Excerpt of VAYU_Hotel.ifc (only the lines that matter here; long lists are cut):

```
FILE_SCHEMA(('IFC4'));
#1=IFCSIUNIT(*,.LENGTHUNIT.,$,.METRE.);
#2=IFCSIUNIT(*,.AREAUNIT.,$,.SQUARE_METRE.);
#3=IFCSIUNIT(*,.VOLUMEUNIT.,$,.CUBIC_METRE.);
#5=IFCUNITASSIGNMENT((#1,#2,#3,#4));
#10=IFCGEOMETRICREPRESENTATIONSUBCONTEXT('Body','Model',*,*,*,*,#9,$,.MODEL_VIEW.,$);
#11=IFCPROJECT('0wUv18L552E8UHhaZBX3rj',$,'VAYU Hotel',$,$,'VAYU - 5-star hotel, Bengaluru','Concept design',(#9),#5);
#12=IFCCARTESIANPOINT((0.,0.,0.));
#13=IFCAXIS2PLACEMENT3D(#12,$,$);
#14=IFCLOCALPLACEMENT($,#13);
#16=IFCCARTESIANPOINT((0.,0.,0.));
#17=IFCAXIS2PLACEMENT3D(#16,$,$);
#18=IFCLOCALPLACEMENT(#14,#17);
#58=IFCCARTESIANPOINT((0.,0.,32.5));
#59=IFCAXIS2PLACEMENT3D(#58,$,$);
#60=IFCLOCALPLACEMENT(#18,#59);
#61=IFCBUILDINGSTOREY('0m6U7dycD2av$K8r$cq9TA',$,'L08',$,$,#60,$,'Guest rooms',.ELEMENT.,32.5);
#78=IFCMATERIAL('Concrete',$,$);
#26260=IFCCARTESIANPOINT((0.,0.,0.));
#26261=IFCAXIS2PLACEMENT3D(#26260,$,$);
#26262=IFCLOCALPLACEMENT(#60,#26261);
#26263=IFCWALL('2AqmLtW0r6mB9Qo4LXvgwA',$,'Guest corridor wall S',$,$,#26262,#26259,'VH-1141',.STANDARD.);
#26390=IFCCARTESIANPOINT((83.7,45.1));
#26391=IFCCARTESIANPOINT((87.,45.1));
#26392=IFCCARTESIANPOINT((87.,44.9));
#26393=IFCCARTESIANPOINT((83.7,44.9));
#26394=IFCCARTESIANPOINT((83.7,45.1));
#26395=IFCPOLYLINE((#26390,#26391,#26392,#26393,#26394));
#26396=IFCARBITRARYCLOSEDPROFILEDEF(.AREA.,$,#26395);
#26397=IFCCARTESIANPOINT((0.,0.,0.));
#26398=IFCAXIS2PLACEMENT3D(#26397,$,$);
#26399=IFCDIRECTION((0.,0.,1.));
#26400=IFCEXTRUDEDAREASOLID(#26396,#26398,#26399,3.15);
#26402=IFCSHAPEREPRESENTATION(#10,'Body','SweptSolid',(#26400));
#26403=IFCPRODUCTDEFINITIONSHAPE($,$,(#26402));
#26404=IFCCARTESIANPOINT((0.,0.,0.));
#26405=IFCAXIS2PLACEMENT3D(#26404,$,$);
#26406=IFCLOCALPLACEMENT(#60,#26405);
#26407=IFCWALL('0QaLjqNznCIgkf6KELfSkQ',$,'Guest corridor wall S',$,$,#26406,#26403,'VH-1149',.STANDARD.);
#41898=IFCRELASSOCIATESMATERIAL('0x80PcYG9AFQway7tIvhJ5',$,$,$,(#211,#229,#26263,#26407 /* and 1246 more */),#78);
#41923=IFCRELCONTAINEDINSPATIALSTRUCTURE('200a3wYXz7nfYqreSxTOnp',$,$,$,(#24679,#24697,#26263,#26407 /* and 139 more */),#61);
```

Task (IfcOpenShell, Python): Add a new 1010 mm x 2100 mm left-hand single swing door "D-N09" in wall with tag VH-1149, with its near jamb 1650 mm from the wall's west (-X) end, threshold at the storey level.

```python
import numpy as np
import ifcopenshell
import ifcopenshell.api.feature
import ifcopenshell.api.geometry
import ifcopenshell.api.root
import ifcopenshell.api.spatial
import ifcopenshell.geom
import ifcopenshell.util.element
import ifcopenshell.util.placement
import ifcopenshell.util.representation
import ifcopenshell.util.shape
import ifcopenshell.util.unit

model = ifcopenshell.open("VAYU_Hotel.ifc")
unit_scale = ifcopenshell.util.unit.calculate_unit_scale(model)
settings = ifcopenshell.geom.settings()


def volume(element):
    """Net volume in cubic metres, openings subtracted."""
    shape = ifcopenshell.geom.create_shape(settings, element)
    return ifcopenshell.util.shape.get_volume(shape.geometry)


wall = model.by_guid("0QaLjqNznCIgkf6KELfSkQ")
storey = ifcopenshell.util.element.get_container(wall, ifc_class="IfcBuildingStorey")
context = ifcopenshell.util.representation.get_context(model, "Model", "Body", "MODEL_VIEW")
before = volume(wall)

width, height, from_end, sill = 1.01, 2.1, 1.65, 0.0  # metres

# The wall runs along its own X axis, and the end named is its -X end.
wall_shape = ifcopenshell.geom.create_shape(settings, wall)
x, y, z = ifcopenshell.util.shape.get_vertices(wall_shape.geometry).T
start = x.min() + from_end
face, thickness = float(y.min()), float(y.max() - y.min())
wall_matrix = ifcopenshell.util.placement.get_local_placement(wall.ObjectPlacement)
level = ifcopenshell.util.placement.get_local_placement(storey.ObjectPlacement)[2, 3]


def in_wall(x, y):
    """Placement at x, y metres in the wall's axes, at sill height."""
    matrix = wall_matrix.copy()
    matrix[:, 3] = wall_matrix @ np.array([x / unit_scale, y / unit_scale, 0.0, 1.0])
    matrix[2, 3] = level + sill / unit_scale
    return matrix


# Opening: a box that overshoots both wall faces by 50 mm.
opening = ifcopenshell.api.root.create_entity(model, ifc_class="IfcOpeningElement", predefined_type="OPENING")
box = ifcopenshell.api.geometry.add_wall_representation(
    model, context=context, length=width, height=height, thickness=thickness + 0.1
)
ifcopenshell.api.geometry.assign_representation(model, product=opening, representation=box)
ifcopenshell.api.geometry.edit_object_placement(model, product=opening, matrix=in_wall(start, face - 0.05), is_si=False)
ifcopenshell.api.feature.add_feature(model, feature=opening, element=wall)

door = ifcopenshell.api.root.create_entity(model, ifc_class="IfcDoor", name="D-N09", predefined_type="DOOR")
door.OverallWidth, door.OverallHeight = width / unit_scale, height / unit_scale
door.OperationType = "SINGLE_SWING_LEFT"
body = ifcopenshell.api.geometry.add_door_representation(
    model,
    context=context,
    overall_width=door.OverallWidth,
    overall_height=door.OverallHeight,
    operation_type="SINGLE_SWING_LEFT",
    lining_properties={"LiningDepth": thickness / unit_scale, "ThresholdDepth": thickness / unit_scale},
)
ifcopenshell.api.geometry.assign_representation(model, product=door, representation=body)
ifcopenshell.api.spatial.assign_container(model, products=[door], relating_structure=storey)
ifcopenshell.api.feature.add_filling(model, opening=opening, element=door)

# The lining spans the wall, so the door starts at the wall face.
ifcopenshell.api.geometry.edit_object_placement(model, product=door, matrix=in_wall(start, face), is_si=False)

after = volume(wall)

print(f"wall volume {before:.3f} -> {after:.3f} m3")

model.write("VAYU_Hotel_edited.ifc")
```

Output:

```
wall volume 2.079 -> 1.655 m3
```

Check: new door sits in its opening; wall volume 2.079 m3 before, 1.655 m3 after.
